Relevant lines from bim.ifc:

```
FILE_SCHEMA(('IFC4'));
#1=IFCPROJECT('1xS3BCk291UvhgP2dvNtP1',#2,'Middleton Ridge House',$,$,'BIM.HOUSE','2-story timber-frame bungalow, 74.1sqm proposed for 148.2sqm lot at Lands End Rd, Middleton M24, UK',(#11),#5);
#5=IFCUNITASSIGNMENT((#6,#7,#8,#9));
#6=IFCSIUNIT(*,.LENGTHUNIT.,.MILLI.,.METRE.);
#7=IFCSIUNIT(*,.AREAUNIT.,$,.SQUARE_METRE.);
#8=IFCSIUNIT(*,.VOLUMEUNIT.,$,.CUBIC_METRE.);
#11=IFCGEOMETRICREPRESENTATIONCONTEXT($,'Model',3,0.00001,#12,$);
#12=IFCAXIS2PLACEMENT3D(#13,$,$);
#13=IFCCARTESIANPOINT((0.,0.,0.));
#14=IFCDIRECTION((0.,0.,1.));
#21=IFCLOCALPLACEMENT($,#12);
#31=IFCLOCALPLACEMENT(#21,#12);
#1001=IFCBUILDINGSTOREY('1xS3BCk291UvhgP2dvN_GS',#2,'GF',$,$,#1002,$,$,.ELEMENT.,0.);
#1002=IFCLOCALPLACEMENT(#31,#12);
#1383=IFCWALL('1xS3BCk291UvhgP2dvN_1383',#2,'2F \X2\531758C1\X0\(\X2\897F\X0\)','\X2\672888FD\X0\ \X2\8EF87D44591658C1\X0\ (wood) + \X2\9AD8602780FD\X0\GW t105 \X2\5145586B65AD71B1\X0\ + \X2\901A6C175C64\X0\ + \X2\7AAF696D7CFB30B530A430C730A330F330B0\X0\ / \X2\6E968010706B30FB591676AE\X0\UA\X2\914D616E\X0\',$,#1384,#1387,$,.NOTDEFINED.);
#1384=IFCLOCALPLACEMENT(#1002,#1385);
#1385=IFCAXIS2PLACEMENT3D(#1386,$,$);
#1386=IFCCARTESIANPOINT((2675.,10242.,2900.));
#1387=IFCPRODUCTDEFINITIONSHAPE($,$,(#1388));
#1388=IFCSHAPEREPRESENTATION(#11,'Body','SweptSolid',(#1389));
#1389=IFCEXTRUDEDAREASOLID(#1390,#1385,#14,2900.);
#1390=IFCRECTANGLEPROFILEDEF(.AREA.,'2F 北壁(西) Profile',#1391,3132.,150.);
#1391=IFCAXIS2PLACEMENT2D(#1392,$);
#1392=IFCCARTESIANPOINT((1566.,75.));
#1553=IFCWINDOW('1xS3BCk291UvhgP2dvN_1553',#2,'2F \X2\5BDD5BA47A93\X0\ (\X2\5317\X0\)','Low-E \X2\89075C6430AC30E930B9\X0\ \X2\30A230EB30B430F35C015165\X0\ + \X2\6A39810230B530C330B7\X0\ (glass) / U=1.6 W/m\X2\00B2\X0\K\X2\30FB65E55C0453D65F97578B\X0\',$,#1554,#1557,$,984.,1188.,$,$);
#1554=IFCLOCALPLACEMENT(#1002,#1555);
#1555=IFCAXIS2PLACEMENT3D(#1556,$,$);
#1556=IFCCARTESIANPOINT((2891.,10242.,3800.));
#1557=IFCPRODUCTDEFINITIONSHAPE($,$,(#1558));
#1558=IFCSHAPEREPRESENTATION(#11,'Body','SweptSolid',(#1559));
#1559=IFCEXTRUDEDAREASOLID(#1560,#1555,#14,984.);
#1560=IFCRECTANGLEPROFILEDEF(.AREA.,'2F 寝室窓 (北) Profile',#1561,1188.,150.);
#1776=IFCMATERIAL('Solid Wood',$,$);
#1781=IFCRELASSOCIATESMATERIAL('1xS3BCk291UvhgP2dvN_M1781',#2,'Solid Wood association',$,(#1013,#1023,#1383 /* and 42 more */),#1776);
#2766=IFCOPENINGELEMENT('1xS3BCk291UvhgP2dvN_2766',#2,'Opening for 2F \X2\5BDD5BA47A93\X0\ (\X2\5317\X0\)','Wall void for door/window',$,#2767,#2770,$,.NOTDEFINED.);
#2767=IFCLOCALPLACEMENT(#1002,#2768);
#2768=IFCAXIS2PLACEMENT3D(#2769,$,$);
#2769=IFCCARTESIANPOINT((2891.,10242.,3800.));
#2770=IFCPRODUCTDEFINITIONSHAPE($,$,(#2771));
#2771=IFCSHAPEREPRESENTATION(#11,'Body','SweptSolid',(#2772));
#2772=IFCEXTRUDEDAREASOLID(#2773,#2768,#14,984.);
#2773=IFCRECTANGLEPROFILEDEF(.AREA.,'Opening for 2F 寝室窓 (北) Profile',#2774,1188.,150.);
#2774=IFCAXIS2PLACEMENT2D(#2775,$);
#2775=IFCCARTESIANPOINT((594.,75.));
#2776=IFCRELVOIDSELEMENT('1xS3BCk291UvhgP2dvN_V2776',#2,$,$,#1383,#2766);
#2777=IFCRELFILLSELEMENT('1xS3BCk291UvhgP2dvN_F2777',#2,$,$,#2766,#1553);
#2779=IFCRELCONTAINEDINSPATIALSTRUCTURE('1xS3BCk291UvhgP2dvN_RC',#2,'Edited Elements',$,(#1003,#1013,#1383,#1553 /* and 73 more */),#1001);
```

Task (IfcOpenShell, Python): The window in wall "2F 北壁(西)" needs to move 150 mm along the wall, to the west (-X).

```python
import ifcopenshell
import ifcopenshell.api.geometry
import ifcopenshell.util.placement
import ifcopenshell.util.unit

model = ifcopenshell.open("bim.ifc")
unit_scale = ifcopenshell.util.unit.calculate_unit_scale(model)

window = model.by_id(1553)
opening = window.FillsVoids[0].RelatingOpeningElement
wall = opening.VoidsElements[0].RelatingBuildingElement

wall_matrix = ifcopenshell.util.placement.get_local_placement(wall.ObjectPlacement)
shift = wall_matrix[:3, 0] * -0.15 / unit_scale
before = ifcopenshell.util.placement.get_local_placement(window.ObjectPlacement)[:3, 3].copy()

# The window is not placed relative to its opening, so move both.
for product in (opening, window):
    matrix = ifcopenshell.util.placement.get_local_placement(product.ObjectPlacement)
    matrix[:3, 3] += shift
    ifcopenshell.api.geometry.edit_object_placement(model, product=product, matrix=matrix, is_si=False)

after = ifcopenshell.util.placement.get_local_placement(window.ObjectPlacement)[:3, 3]
print("window moved by", (after - before).round(3) + 0.0)

model.write("bim_edited.ifc")
```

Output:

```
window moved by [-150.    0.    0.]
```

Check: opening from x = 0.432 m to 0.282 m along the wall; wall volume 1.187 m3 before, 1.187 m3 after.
